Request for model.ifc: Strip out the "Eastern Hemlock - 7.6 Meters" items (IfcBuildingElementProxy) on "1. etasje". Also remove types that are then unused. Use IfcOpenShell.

First a look at what the model holds.

```python
import ifcopenshell
import ifcopenshell.util.element

model = ifcopenshell.open("model.ifc")
print(model.schema)
storey = next(s for s in model.by_type("IfcBuildingStorey") if s.Name == "1. etasje")
proxies = [e for e in ifcopenshell.util.element.get_decomposition(storey) if e.is_a("IfcBuildingElementProxy")]
seen = {}
for e in proxies:
    element_type = ifcopenshell.util.element.get_type(e)
    name = element_type.Name if element_type not in (None, e) else None
    seen[name] = seen.get(name, 0) + 1
for name, count in sorted(seen.items(), key=str):
    print(count, "x", name)
```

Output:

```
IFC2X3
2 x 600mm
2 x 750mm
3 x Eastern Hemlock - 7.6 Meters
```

```python
import ifcopenshell
import ifcopenshell.api.root
import ifcopenshell.util.element

model = ifcopenshell.open("model.ifc")

storey = next(s for s in model.by_type("IfcBuildingStorey") if s.Name == "1. etasje")
proxies = [e for e in ifcopenshell.util.element.get_decomposition(storey) if e.is_a("IfcBuildingElementProxy")]
targets = [e for e in proxies if (t := ifcopenshell.util.element.get_type(e)) not in (None, e) and t.Name == "Eastern Hemlock - 7.6 Meters"]
types = {ifcopenshell.util.element.get_type(e) for e in targets} - {None, *targets}

for e in targets:
    ifcopenshell.api.root.remove_product(model, product=e)
print(len(targets), "removed")

unused = [t for t in types if not ifcopenshell.util.element.get_types(t)]
for t in unused:
    ifcopenshell.api.root.remove_product(model, product=t)
print(len(unused), "unused types removed")

model.write("model_rev.ifc")
```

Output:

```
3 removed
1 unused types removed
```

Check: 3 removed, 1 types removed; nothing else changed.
